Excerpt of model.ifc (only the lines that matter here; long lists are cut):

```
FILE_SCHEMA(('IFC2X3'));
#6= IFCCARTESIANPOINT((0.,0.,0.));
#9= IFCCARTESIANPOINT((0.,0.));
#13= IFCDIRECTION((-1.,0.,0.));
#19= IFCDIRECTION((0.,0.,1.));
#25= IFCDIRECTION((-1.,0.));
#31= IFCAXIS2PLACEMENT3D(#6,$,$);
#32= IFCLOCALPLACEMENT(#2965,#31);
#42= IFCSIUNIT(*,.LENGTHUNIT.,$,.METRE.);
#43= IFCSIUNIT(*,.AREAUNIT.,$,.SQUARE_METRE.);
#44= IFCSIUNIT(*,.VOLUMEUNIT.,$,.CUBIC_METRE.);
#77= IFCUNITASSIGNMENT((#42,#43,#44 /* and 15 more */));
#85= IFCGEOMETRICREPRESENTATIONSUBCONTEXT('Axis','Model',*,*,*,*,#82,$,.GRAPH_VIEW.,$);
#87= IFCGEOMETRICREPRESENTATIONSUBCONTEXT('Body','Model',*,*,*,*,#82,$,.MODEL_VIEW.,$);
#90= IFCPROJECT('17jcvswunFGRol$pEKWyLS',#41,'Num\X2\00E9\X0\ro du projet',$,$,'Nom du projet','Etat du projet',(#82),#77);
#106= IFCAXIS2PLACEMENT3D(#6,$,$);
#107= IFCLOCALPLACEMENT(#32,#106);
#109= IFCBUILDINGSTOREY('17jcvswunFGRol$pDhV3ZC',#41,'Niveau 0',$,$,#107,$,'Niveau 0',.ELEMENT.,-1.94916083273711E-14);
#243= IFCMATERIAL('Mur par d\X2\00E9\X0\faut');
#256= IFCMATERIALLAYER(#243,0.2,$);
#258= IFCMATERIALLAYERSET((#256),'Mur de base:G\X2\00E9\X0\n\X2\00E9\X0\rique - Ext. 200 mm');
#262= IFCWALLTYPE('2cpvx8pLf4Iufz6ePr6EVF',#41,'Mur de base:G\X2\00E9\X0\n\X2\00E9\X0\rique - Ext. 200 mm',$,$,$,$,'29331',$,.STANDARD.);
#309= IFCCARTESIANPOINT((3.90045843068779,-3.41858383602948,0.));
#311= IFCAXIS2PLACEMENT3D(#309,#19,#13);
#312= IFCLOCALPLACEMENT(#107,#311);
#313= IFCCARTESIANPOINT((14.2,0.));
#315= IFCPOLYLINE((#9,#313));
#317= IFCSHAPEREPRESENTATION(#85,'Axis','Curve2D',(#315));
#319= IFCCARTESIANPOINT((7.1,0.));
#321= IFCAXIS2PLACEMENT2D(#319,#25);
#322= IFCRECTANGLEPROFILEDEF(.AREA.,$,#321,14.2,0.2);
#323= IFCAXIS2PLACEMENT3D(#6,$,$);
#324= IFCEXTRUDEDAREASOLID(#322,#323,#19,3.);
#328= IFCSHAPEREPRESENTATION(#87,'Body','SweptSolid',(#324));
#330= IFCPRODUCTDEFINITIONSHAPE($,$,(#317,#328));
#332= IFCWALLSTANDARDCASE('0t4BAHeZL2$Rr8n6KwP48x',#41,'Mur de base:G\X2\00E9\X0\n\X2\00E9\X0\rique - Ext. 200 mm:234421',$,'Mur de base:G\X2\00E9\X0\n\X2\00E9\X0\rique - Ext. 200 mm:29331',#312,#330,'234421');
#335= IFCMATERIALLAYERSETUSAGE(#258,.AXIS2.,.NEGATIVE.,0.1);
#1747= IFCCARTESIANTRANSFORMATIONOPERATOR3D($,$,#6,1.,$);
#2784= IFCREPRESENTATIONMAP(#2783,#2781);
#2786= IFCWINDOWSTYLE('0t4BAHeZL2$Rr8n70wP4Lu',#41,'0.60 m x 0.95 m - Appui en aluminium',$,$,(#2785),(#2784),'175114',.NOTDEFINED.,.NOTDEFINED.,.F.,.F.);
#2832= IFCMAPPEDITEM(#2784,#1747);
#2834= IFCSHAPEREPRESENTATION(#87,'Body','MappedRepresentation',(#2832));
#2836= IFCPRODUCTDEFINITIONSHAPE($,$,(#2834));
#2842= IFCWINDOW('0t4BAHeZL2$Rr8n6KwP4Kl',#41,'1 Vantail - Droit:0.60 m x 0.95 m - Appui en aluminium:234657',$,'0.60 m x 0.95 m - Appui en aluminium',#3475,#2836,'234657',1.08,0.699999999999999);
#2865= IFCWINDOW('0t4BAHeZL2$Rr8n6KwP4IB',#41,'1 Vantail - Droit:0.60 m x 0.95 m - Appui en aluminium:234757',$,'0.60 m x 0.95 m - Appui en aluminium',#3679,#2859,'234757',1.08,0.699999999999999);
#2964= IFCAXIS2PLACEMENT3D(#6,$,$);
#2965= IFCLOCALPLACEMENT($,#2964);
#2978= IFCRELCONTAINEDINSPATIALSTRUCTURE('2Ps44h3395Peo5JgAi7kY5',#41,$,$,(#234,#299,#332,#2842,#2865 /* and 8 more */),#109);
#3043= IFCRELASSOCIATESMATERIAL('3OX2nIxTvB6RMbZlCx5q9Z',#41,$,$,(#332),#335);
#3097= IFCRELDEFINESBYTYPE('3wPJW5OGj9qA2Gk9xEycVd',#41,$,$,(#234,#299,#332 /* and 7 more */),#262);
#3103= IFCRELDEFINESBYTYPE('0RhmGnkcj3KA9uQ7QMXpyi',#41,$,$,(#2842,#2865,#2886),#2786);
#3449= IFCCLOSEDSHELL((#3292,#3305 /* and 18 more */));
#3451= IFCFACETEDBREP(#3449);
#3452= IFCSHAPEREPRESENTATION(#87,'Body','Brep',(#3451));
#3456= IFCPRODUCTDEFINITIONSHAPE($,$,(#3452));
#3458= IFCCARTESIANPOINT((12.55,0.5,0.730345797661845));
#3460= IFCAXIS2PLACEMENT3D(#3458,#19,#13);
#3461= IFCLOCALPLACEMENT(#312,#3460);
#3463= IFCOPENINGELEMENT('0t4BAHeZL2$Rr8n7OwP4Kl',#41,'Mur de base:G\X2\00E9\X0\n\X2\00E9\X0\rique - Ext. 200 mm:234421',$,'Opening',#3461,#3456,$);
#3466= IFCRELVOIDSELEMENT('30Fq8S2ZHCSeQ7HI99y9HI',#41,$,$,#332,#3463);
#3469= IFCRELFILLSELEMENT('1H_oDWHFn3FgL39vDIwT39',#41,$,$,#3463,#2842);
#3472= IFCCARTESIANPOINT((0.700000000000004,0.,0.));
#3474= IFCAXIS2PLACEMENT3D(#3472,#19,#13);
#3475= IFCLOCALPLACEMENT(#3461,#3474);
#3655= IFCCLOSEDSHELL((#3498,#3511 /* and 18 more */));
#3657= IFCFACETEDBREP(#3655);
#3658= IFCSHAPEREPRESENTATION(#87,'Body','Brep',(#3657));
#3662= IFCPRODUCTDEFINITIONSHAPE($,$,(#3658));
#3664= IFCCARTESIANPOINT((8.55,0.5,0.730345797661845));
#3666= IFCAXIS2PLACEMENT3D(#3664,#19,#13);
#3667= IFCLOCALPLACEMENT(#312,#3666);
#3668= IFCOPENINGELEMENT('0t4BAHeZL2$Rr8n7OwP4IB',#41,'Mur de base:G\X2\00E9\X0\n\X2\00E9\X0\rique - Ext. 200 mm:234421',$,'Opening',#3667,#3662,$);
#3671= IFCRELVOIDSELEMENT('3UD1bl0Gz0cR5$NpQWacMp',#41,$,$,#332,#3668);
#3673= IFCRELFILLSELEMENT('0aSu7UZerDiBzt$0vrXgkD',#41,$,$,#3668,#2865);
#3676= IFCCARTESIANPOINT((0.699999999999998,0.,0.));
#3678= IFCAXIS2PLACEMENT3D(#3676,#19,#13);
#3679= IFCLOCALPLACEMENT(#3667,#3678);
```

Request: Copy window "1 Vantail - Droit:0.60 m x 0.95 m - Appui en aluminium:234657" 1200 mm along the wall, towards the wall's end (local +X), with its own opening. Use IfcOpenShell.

```python
import ifcopenshell
import ifcopenshell.api.feature
import ifcopenshell.api.geometry
import ifcopenshell.api.root
import ifcopenshell.geom
import ifcopenshell.util.element
import ifcopenshell.util.placement
import ifcopenshell.util.shape
import ifcopenshell.util.unit

model = ifcopenshell.open("model.ifc")
unit_scale = ifcopenshell.util.unit.calculate_unit_scale(model)
settings = ifcopenshell.geom.settings()


def volume(element):
    """Net volume in cubic metres, openings subtracted."""
    shape = ifcopenshell.geom.create_shape(settings, element)
    return ifcopenshell.util.shape.get_volume(shape.geometry)


def reuse_history(source, copy):
    """copy_class also copies each property set's owner history, people and application; keep the originals."""
    for rel in copy.IsDefinedBy:
        if rel.is_a("IfcRelDefinesByProperties") and (history := rel.RelatingPropertyDefinition.OwnerHistory):
            rel.RelatingPropertyDefinition.OwnerHistory = source.OwnerHistory
            ifcopenshell.util.element.remove_deep2(model, history)


window = model.by_id(2842)
opening = window.FillsVoids[0].RelatingOpeningElement
wall = opening.VoidsElements[0].RelatingBuildingElement
before = volume(wall)
shift = ifcopenshell.util.placement.get_local_placement(wall.ObjectPlacement)[:3, 0] * 1.2 / unit_scale

# copy_class copies the void relationship, type, container and properties, but no geometry.
new_opening = ifcopenshell.api.root.copy_class(model, product=opening)
new_opening.Representation = ifcopenshell.util.element.copy_deep(
    model, opening.Representation, exclude=["IfcGeometricRepresentationContext", "IfcRepresentationMap"]
)
new_opening.Name = "Mur de base:Générique - Ext. 200 mm"
new_window = ifcopenshell.api.root.copy_class(model, product=window)
new_window.Representation = ifcopenshell.util.element.copy_deep(
    model, window.Representation, exclude=["IfcGeometricRepresentationContext", "IfcRepresentationMap"]
)
new_window.Name = "1 Vantail - Droit:0.60 m x 0.95 m - Appui en aluminium"
new_window.Tag = None
reuse_history(window, new_window)
fills = ifcopenshell.api.feature.add_filling(model, opening=new_opening, element=new_window)
fills.OwnerHistory = new_window.OwnerHistory  # required in IFC2X3

for old, new in ((opening, new_opening), (window, new_window)):
    matrix = ifcopenshell.util.placement.get_local_placement(old.ObjectPlacement)
    matrix[:3, 3] += shift
    ifcopenshell.api.geometry.edit_object_placement(model, product=new, matrix=matrix, is_si=False)

after = volume(wall)

print(f"wall volume {before:.3f} -> {after:.3f} m3")

model.write("model_updated.ifc")
```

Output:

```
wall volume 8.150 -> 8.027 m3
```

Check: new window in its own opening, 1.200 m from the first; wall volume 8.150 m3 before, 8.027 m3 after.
